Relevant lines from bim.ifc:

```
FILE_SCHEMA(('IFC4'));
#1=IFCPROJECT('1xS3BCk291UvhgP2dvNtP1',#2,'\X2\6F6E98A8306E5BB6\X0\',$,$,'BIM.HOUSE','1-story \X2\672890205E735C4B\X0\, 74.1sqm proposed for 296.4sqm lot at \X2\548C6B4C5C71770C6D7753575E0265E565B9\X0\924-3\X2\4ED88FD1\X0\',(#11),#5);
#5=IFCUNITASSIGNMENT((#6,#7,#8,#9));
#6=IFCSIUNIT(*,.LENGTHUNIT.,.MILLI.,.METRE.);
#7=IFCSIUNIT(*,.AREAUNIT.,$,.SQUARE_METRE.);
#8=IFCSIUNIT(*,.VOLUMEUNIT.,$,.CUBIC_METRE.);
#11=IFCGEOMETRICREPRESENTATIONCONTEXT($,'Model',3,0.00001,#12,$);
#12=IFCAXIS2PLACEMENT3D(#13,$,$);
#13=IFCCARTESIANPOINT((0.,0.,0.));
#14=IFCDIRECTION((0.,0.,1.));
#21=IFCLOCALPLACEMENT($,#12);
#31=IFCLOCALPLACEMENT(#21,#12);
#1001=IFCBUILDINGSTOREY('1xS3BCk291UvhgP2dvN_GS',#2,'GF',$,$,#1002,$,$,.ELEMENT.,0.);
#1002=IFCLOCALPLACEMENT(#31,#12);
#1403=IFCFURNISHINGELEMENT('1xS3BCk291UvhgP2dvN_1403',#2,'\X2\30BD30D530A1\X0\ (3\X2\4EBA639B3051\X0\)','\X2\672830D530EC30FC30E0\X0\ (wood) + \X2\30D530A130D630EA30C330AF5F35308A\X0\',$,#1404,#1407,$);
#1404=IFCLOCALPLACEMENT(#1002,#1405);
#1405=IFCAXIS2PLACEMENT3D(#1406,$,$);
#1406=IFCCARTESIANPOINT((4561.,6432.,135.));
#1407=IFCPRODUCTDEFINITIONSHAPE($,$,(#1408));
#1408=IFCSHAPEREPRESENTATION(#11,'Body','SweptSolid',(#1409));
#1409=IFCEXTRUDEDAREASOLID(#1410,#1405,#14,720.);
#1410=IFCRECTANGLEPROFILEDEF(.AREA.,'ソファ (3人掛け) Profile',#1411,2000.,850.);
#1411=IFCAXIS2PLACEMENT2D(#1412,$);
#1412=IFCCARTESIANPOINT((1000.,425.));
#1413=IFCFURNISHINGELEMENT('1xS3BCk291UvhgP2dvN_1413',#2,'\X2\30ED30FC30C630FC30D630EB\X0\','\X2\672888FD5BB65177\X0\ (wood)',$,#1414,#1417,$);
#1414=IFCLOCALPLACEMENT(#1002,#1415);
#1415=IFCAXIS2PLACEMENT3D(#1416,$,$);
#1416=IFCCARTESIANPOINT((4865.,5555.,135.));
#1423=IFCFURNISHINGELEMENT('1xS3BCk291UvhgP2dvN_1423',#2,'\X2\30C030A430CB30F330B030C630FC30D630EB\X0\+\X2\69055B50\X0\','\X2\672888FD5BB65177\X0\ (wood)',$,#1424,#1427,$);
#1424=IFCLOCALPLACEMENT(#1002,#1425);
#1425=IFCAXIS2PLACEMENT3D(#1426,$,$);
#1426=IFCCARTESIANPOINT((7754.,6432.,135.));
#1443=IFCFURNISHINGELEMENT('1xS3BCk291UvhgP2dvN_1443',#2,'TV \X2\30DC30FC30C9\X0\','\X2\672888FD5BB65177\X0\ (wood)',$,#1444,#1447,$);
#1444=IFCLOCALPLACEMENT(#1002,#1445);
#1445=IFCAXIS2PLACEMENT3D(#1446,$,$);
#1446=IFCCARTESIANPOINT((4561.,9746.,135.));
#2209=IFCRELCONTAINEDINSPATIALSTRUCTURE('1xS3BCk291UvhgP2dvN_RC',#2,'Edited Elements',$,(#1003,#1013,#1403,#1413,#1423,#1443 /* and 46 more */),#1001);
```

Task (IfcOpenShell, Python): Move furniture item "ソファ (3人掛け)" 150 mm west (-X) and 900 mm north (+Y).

```python
import ifcopenshell
import ifcopenshell.api.geometry
import ifcopenshell.util.placement

model = ifcopenshell.open("bim.ifc")

item = model.by_guid("1xS3BCk291UvhgP2dvN_1403")
matrix = ifcopenshell.util.placement.get_local_placement(item.ObjectPlacement)
matrix[0, 3] -= 150.0
matrix[1, 3] += 900.0
ifcopenshell.api.geometry.edit_object_placement(model, product=item, matrix=matrix, is_si=False)

print(ifcopenshell.util.placement.get_local_placement(item.ObjectPlacement).round(3) + 0.0)

model.write("bim_v2.ifc")
```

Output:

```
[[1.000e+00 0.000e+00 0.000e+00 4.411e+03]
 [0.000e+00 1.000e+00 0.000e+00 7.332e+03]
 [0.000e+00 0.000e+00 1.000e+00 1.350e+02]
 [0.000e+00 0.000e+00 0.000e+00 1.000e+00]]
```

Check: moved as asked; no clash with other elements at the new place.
